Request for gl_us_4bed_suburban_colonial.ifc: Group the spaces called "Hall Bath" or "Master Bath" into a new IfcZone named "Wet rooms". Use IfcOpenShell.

First a look at what the model holds.

```python
import ifcopenshell

model = ifcopenshell.open("gl_us_4bed_suburban_colonial.ifc")
print(model.schema)
seen = {}
for space in model.by_type("IfcSpace"):
    seen[space.LongName] = seen.get(space.LongName, 0) + 1
for name, count in sorted(seen.items(), key=str):
    print(count, "x", name)
print("zones:", [z.Name for z in model.by_type("IfcZone")][:20])
```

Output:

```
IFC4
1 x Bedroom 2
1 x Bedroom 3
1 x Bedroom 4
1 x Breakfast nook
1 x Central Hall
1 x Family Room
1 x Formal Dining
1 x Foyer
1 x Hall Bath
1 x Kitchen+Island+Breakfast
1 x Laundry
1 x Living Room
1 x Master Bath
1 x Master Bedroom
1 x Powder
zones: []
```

```python
import ifcopenshell
import ifcopenshell.api.group
import ifcopenshell.api.root

model = ifcopenshell.open("gl_us_4bed_suburban_colonial.ifc")

names = {"Hall Bath", "Master Bath"}
spaces = [s for s in model.by_type("IfcSpace") if s.LongName in names]

zone = ifcopenshell.api.root.create_entity(model, ifc_class="IfcZone", name="Wet rooms")
ifcopenshell.api.group.assign_group(model, products=spaces, group=zone)
print(len(spaces), "spaces in", zone.Name)

model.write("gl_us_4bed_suburban_colonial_rev.ifc")
```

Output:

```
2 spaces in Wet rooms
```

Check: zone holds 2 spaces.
